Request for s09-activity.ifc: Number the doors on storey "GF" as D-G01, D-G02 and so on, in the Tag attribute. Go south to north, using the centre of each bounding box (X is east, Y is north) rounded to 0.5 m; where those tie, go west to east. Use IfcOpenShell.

First a look at what the model holds.

```python
import ifcopenshell
import ifcopenshell.util.element
import ifcopenshell.util.placement

model = ifcopenshell.open("s09-activity.ifc")
print(model.schema)
storey = next(s for s in model.by_type("IfcBuildingStorey") if s.Name == "GF")
doors = [e for e in ifcopenshell.util.element.get_decomposition(storey) if e.is_a("IfcDoor")]
for e in sorted(doors, key=lambda e: e.id()):
    origin = ifcopenshell.util.placement.get_local_placement(e.ObjectPlacement)[:3, 3]
    print(e.id(), e.Tag, e.Name, origin.round(2) + 0.0, sep=" | ")
```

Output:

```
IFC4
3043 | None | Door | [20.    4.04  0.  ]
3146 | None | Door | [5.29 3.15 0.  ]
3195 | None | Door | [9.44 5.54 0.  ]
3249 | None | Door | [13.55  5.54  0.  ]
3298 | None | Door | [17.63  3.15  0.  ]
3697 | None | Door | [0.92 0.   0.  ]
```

```python
import ifcopenshell
import ifcopenshell.geom
import ifcopenshell.util.element
import ifcopenshell.util.shape

model = ifcopenshell.open("s09-activity.ifc")
settings = ifcopenshell.geom.settings()
settings.set("use-world-coords", True)


def centre(element):
    shape = ifcopenshell.geom.create_shape(settings, element)
    return ifcopenshell.util.shape.get_bbox_centroid(shape.geometry)


storey = next(s for s in model.by_type("IfcBuildingStorey") if s.Name == "GF")
doors = [e for e in ifcopenshell.util.element.get_decomposition(storey) if e.is_a("IfcDoor")]

# Insertion points can sit at a corner or the storey origin, so sort by the geometry (in metres).
centres = {e: centre(e) for e in doors}
doors.sort(key=lambda e: (round(centres[e][1] / 0.5), centres[e][0]))

for i, e in enumerate(doors, start=1):
    number = f"D-G{i:02d}"
    e.Tag = number
    print(e.id(), number)

model.write("s09-activity_rev.ifc")
```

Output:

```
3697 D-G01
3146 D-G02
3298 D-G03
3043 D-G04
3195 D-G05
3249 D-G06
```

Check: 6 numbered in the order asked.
